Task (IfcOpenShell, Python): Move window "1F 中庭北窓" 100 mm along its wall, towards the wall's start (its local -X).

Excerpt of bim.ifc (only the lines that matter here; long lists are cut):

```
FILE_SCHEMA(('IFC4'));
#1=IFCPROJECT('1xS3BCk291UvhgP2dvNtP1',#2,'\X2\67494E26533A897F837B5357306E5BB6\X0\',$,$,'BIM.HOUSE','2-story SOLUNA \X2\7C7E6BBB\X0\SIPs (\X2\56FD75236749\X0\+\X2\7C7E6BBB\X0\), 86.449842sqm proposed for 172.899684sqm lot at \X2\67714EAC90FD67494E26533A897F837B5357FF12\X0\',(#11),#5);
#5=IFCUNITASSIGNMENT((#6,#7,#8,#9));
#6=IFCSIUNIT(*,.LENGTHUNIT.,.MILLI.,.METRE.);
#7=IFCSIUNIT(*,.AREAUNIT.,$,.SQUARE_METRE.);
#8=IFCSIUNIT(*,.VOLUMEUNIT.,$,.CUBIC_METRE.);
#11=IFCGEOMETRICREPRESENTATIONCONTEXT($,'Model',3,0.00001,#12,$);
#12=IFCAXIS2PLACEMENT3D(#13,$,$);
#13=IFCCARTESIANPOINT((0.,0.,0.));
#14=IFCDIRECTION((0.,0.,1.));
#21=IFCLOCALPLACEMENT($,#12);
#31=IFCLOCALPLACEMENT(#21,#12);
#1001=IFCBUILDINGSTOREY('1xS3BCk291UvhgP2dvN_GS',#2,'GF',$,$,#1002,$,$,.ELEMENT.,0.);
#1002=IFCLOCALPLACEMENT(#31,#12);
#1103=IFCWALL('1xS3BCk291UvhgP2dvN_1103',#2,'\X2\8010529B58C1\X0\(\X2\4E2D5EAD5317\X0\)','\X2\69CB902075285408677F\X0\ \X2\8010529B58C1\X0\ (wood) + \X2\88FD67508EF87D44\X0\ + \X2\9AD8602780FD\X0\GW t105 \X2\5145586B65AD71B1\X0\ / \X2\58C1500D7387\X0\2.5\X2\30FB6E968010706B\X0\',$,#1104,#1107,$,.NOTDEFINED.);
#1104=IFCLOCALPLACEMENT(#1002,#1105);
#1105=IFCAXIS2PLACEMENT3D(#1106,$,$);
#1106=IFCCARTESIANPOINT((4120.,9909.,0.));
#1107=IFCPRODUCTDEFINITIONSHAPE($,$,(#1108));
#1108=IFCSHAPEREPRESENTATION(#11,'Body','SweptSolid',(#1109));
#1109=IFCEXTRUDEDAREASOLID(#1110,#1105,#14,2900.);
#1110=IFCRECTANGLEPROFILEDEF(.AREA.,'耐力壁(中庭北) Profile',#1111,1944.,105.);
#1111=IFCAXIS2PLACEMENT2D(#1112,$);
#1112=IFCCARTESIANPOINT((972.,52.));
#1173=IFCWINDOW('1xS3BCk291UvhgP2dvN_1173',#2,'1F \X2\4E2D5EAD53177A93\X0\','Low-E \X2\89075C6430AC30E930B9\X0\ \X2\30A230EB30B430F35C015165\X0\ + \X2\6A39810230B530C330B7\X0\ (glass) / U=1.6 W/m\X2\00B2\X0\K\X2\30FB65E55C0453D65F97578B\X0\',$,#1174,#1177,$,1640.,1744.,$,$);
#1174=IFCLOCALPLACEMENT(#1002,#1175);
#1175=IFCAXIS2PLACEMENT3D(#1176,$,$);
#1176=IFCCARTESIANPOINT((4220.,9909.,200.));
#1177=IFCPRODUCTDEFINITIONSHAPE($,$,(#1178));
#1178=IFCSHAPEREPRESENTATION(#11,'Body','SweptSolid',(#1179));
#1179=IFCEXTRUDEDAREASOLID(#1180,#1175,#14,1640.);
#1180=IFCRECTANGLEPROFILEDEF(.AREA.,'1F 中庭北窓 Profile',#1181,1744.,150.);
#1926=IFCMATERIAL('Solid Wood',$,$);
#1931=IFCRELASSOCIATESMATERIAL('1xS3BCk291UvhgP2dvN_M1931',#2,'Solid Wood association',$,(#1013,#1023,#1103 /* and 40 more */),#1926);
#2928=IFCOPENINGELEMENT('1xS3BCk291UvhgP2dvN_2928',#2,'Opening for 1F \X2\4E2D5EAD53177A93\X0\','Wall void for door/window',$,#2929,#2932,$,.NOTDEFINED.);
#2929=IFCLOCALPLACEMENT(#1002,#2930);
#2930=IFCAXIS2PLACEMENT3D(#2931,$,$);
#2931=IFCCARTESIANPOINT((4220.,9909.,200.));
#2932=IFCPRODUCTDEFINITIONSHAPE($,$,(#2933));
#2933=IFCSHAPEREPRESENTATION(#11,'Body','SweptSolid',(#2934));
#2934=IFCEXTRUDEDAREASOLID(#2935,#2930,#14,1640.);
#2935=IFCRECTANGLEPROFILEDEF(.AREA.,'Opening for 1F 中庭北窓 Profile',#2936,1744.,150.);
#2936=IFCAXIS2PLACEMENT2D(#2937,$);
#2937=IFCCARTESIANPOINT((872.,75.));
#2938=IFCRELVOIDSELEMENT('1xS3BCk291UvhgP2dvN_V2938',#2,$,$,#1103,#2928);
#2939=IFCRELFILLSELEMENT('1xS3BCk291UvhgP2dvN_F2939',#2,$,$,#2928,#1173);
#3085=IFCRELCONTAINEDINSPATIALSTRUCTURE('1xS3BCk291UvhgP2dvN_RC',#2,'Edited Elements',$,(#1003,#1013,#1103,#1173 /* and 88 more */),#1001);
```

```python
import ifcopenshell
import ifcopenshell.api.geometry
import ifcopenshell.util.placement
import ifcopenshell.util.unit

model = ifcopenshell.open("bim.ifc")
unit_scale = ifcopenshell.util.unit.calculate_unit_scale(model)

window = model.by_guid("1xS3BCk291UvhgP2dvN_1173")
opening = window.FillsVoids[0].RelatingOpeningElement
wall = opening.VoidsElements[0].RelatingBuildingElement

wall_matrix = ifcopenshell.util.placement.get_local_placement(wall.ObjectPlacement)
shift = wall_matrix[:3, 0] * -0.1 / unit_scale
before = ifcopenshell.util.placement.get_local_placement(window.ObjectPlacement)[:3, 3].copy()

# The window is not placed relative to its opening, so move both.
for product in (opening, window):
    matrix = ifcopenshell.util.placement.get_local_placement(product.ObjectPlacement)
    matrix[:3, 3] += shift
    ifcopenshell.api.geometry.edit_object_placement(model, product=product, matrix=matrix, is_si=False)

after = ifcopenshell.util.placement.get_local_placement(window.ObjectPlacement)[:3, 3]
print("window moved by", (after - before).round(3) + 0.0)

model.write("bim-out.ifc")
```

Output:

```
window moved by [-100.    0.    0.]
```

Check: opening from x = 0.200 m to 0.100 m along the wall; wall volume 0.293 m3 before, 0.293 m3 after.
